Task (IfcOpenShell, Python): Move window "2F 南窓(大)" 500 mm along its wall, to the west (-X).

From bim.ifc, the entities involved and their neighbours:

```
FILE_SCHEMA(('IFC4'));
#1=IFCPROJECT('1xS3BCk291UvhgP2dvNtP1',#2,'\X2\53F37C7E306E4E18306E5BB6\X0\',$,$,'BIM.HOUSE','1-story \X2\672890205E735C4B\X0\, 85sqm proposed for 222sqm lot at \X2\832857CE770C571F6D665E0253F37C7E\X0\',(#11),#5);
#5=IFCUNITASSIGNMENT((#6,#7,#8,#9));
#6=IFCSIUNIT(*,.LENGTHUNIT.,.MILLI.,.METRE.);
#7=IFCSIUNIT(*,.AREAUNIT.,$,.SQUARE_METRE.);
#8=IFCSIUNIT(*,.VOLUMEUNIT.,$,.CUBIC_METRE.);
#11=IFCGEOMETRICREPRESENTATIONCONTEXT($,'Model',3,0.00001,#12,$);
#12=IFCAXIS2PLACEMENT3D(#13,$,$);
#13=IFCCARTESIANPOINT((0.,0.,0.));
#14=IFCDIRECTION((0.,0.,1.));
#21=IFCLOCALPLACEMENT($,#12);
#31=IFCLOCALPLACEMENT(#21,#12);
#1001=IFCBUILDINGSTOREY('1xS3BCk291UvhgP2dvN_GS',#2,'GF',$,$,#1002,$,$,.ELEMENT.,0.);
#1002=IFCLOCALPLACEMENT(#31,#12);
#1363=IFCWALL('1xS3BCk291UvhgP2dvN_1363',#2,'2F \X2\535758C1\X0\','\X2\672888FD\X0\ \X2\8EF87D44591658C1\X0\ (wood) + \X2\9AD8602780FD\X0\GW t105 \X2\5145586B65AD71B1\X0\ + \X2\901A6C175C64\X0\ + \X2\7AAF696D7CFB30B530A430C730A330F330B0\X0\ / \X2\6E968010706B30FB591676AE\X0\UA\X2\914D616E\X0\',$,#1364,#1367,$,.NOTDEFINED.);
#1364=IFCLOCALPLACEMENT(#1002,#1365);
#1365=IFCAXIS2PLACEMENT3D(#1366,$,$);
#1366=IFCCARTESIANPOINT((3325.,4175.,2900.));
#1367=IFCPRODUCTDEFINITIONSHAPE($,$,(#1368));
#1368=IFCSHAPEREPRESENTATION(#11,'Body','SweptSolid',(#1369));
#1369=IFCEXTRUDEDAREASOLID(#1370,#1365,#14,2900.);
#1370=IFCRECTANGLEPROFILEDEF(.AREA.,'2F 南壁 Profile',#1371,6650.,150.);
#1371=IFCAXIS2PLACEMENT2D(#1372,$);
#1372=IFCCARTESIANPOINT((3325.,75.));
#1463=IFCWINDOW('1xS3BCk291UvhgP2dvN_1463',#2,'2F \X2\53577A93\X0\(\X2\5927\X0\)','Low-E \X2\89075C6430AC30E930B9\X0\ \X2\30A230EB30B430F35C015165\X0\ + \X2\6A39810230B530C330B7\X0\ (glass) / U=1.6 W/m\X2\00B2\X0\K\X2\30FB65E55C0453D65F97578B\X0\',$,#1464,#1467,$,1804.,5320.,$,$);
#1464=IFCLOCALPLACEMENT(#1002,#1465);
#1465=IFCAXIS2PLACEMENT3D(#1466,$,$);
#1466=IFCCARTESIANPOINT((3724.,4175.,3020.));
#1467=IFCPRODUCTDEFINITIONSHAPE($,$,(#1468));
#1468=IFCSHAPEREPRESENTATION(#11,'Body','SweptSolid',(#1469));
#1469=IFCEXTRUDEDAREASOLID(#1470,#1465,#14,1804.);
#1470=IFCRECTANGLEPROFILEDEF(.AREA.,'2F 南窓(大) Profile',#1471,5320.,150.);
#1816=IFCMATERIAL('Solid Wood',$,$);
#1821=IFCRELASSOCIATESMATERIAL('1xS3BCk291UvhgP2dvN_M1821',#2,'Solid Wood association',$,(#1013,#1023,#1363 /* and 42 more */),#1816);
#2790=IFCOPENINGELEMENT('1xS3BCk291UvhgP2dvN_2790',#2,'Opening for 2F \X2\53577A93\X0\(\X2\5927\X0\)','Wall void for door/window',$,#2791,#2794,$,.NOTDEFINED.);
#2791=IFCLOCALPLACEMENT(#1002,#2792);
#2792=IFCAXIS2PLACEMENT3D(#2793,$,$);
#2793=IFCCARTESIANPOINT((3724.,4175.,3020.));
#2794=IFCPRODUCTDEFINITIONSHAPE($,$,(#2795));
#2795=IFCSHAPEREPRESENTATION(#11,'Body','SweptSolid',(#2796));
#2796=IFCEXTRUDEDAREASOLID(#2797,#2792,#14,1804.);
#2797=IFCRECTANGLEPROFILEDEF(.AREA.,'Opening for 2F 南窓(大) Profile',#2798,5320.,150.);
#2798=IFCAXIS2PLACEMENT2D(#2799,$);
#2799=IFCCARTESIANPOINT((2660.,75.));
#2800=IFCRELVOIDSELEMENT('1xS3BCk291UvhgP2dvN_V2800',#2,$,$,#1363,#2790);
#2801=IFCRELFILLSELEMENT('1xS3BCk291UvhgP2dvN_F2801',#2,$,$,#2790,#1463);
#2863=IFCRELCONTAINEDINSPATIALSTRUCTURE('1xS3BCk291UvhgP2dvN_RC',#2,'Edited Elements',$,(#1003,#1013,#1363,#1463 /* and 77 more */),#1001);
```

```python
import ifcopenshell
import ifcopenshell.api.geometry
import ifcopenshell.util.placement

model = ifcopenshell.open("bim.ifc")

window = model.by_guid("1xS3BCk291UvhgP2dvN_1463")
opening = window.FillsVoids[0].RelatingOpeningElement
wall = opening.VoidsElements[0].RelatingBuildingElement

wall_matrix = ifcopenshell.util.placement.get_local_placement(wall.ObjectPlacement)
shift = wall_matrix[:3, 0] * -500.0
before = ifcopenshell.util.placement.get_local_placement(window.ObjectPlacement)[:3, 3].copy()

# The window is not placed relative to its opening, so move both.
for product in (opening, window):
    matrix = ifcopenshell.util.placement.get_local_placement(product.ObjectPlacement)
    matrix[:3, 3] += shift
    ifcopenshell.api.geometry.edit_object_placement(model, product=product, matrix=matrix, is_si=False)

after = ifcopenshell.util.placement.get_local_placement(window.ObjectPlacement)[:3, 3]
print("window moved by", (after - before).round(3) + 0.0)

model.write("bim_rev.ifc")
```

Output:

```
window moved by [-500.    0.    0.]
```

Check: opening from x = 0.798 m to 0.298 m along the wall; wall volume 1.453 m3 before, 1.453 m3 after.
